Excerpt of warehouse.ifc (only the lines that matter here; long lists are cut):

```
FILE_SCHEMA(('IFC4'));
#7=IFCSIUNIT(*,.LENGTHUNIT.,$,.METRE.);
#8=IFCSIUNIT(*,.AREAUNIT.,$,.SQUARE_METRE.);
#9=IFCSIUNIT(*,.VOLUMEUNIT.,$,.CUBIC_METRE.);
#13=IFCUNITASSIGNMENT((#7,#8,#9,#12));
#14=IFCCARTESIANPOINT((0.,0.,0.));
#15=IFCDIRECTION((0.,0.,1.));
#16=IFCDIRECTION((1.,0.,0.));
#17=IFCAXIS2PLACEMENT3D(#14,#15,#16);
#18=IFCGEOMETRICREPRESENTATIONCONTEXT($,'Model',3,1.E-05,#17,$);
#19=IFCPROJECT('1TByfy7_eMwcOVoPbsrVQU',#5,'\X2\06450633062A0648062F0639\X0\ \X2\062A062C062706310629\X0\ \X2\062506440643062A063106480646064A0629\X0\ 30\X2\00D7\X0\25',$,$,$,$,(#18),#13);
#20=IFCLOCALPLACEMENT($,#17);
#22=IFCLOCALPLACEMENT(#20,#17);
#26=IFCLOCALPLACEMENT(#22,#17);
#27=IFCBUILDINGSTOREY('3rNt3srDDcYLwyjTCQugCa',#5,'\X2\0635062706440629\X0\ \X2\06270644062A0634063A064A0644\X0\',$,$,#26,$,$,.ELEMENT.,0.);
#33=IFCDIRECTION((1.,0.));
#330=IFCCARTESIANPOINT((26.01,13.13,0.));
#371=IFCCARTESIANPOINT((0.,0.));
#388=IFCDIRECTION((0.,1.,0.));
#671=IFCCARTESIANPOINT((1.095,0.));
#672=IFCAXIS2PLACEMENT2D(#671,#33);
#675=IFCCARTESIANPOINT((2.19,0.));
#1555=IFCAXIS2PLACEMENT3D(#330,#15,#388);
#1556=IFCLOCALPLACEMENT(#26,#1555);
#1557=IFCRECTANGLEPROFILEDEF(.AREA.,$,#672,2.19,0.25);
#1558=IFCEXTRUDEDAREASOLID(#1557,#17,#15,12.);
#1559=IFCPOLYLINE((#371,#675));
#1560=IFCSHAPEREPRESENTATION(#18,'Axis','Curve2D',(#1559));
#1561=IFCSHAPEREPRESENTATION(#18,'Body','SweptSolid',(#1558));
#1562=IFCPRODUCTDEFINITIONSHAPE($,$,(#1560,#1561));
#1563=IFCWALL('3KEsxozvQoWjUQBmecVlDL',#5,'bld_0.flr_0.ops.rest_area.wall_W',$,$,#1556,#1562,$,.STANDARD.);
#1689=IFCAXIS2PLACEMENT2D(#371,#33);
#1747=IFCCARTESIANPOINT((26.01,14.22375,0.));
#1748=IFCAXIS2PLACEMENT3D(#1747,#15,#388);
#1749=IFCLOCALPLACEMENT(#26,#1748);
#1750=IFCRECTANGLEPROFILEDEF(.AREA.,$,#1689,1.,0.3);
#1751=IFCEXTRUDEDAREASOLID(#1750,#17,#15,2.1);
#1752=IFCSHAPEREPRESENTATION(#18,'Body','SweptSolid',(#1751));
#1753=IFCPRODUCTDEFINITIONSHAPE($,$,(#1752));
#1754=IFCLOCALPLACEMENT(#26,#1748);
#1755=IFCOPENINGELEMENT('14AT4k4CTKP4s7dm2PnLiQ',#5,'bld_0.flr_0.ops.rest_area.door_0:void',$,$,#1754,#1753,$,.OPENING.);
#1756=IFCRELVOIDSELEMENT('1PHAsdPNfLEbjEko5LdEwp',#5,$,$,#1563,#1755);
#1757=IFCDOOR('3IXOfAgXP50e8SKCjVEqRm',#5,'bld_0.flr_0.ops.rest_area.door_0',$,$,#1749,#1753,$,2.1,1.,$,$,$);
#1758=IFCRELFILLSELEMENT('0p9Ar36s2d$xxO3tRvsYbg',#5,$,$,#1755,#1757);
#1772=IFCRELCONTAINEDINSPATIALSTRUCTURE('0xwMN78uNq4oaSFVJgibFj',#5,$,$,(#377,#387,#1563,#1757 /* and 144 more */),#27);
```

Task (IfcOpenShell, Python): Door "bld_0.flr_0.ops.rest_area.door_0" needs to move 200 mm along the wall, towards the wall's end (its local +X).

```python
import ifcopenshell
import ifcopenshell.api.geometry
import ifcopenshell.util.placement

model = ifcopenshell.open("warehouse.ifc")

door = model.by_guid("3IXOfAgXP50e8SKCjVEqRm")
opening = door.FillsVoids[0].RelatingOpeningElement
wall = opening.VoidsElements[0].RelatingBuildingElement

wall_matrix = ifcopenshell.util.placement.get_local_placement(wall.ObjectPlacement)
shift = wall_matrix[:3, 0] * 0.2
before = ifcopenshell.util.placement.get_local_placement(door.ObjectPlacement)[:3, 3].copy()

# The door is not placed relative to its opening, so move both.
for product in (opening, door):
    matrix = ifcopenshell.util.placement.get_local_placement(product.ObjectPlacement)
    matrix[:3, 3] += shift
    ifcopenshell.api.geometry.edit_object_placement(model, product=product, matrix=matrix, is_si=False)

after = ifcopenshell.util.placement.get_local_placement(door.ObjectPlacement)[:3, 3]
print("door moved by", (after - before).round(3) + 0.0)

model.write("warehouse_edited.ifc")
```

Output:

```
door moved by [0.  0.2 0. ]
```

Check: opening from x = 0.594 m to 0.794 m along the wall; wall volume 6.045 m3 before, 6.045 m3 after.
